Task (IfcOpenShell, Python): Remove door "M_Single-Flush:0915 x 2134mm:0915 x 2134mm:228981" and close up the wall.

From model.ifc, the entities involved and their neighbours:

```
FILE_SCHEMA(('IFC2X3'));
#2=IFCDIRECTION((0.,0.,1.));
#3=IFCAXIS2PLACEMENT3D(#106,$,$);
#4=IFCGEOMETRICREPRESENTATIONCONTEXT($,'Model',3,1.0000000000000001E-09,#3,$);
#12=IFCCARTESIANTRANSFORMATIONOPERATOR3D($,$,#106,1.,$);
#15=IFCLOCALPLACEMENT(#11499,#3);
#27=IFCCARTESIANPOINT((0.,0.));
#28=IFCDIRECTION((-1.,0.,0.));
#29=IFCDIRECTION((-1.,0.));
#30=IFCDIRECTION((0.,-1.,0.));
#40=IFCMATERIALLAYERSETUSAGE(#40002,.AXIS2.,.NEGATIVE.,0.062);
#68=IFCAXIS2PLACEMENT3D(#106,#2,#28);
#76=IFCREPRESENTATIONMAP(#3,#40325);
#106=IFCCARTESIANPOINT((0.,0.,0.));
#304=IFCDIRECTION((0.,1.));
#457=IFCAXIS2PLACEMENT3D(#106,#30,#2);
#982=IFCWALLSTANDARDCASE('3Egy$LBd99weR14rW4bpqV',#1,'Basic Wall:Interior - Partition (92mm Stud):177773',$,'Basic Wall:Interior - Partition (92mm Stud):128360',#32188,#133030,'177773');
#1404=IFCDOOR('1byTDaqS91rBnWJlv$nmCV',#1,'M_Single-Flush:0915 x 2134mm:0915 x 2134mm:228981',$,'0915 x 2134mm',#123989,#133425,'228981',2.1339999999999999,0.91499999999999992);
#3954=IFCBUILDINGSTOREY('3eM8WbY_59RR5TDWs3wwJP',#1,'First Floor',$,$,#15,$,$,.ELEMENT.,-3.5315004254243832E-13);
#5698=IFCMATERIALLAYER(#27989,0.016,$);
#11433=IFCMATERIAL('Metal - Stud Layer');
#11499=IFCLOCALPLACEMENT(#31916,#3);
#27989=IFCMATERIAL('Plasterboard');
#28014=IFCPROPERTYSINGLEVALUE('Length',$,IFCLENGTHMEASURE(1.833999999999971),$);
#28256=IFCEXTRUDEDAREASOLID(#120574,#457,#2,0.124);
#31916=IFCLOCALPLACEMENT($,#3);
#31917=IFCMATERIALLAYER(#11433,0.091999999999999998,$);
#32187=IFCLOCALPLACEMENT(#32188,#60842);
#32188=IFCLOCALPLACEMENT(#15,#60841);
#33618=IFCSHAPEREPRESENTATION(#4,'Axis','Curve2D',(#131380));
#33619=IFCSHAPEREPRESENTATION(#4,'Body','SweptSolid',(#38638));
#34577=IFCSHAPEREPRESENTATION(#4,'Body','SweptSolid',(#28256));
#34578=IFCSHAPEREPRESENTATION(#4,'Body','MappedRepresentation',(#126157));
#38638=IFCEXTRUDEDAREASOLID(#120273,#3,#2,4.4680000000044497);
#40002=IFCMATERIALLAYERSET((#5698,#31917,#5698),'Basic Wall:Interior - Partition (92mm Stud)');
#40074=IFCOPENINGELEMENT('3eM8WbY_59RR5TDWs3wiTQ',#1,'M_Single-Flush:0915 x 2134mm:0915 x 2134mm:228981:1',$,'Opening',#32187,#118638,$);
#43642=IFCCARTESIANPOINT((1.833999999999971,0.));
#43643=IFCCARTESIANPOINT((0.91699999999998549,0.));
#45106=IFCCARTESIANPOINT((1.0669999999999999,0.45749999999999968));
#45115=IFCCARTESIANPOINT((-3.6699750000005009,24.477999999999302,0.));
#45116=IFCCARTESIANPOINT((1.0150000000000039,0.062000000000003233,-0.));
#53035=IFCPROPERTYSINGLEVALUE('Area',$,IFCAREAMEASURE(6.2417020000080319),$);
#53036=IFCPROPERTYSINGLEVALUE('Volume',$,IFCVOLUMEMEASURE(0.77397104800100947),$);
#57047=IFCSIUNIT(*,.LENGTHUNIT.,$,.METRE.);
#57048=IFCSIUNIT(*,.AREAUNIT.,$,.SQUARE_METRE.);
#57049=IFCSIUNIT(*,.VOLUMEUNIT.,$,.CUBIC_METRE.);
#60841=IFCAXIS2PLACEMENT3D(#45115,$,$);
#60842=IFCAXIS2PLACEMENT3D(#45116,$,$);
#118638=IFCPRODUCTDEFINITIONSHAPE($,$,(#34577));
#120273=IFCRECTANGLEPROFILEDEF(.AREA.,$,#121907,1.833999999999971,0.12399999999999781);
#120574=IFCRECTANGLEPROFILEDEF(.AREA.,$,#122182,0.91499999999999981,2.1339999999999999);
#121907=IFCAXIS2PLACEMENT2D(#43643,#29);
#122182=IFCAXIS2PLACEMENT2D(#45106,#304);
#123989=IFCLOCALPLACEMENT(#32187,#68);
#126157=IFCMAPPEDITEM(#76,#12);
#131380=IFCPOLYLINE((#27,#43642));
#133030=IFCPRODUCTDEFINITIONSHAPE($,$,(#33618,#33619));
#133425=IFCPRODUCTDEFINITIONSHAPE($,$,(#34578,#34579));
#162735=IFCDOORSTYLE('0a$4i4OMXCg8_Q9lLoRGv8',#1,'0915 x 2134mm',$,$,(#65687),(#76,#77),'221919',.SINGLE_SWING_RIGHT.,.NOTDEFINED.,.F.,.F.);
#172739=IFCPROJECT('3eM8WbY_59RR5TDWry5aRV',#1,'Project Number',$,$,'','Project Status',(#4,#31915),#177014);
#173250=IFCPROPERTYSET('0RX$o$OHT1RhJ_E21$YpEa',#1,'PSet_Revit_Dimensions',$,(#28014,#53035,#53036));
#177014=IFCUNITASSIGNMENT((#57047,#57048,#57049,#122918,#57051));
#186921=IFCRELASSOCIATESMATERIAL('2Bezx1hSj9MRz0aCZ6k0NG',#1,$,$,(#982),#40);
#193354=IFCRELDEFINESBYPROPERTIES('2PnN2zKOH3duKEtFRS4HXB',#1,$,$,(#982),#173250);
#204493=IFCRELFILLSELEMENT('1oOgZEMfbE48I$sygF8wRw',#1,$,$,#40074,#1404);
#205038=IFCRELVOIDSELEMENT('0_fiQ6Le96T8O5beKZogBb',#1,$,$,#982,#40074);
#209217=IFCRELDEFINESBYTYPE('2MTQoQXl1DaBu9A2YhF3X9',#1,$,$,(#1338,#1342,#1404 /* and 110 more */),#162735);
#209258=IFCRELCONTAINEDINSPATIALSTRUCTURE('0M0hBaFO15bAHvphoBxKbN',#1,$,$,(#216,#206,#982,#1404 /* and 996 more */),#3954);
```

```python
import ifcopenshell
import ifcopenshell.api.feature
import ifcopenshell.api.pset
import ifcopenshell.api.root
import ifcopenshell.geom
import ifcopenshell.util.element
import ifcopenshell.util.shape
import ifcopenshell.util.unit

model = ifcopenshell.open("model.ifc")
area_scale = ifcopenshell.util.unit.calculate_unit_scale(model, "AREAUNIT")
volume_scale = ifcopenshell.util.unit.calculate_unit_scale(model, "VOLUMEUNIT")
settings = ifcopenshell.geom.settings()


def volume(element):
    """Net volume in cubic metres, openings subtracted."""
    shape = ifcopenshell.geom.create_shape(settings, element)
    return ifcopenshell.util.shape.get_volume(shape.geometry)


door = model.by_guid("1byTDaqS91rBnWJlv$nmCV")
opening = door.FillsVoids[0].RelatingOpeningElement
wall = opening.VoidsElements[0].RelatingBuildingElement
before = volume(wall)

ifcopenshell.api.root.remove_product(model, product=door)
ifcopenshell.api.feature.remove_feature(model, feature=opening)

after = volume(wall)
thickness = 0.124  # wall thickness in metres

# Update the wall's stored quantities.
pset = model.by_id(ifcopenshell.util.element.get_pset(wall, "PSet_Revit_Dimensions", should_inherit=False)["id"])
ifcopenshell.api.pset.edit_pset(model, pset=pset, properties={
    "Area": model.create_entity("IfcAreaMeasure", after / thickness / area_scale),
    "Volume": model.create_entity("IfcVolumeMeasure", after / volume_scale),
})

print(f"wall volume {before:.3f} -> {after:.3f} m3")

model.write("model-out.ifc")
```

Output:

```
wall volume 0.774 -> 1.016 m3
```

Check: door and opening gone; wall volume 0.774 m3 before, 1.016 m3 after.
